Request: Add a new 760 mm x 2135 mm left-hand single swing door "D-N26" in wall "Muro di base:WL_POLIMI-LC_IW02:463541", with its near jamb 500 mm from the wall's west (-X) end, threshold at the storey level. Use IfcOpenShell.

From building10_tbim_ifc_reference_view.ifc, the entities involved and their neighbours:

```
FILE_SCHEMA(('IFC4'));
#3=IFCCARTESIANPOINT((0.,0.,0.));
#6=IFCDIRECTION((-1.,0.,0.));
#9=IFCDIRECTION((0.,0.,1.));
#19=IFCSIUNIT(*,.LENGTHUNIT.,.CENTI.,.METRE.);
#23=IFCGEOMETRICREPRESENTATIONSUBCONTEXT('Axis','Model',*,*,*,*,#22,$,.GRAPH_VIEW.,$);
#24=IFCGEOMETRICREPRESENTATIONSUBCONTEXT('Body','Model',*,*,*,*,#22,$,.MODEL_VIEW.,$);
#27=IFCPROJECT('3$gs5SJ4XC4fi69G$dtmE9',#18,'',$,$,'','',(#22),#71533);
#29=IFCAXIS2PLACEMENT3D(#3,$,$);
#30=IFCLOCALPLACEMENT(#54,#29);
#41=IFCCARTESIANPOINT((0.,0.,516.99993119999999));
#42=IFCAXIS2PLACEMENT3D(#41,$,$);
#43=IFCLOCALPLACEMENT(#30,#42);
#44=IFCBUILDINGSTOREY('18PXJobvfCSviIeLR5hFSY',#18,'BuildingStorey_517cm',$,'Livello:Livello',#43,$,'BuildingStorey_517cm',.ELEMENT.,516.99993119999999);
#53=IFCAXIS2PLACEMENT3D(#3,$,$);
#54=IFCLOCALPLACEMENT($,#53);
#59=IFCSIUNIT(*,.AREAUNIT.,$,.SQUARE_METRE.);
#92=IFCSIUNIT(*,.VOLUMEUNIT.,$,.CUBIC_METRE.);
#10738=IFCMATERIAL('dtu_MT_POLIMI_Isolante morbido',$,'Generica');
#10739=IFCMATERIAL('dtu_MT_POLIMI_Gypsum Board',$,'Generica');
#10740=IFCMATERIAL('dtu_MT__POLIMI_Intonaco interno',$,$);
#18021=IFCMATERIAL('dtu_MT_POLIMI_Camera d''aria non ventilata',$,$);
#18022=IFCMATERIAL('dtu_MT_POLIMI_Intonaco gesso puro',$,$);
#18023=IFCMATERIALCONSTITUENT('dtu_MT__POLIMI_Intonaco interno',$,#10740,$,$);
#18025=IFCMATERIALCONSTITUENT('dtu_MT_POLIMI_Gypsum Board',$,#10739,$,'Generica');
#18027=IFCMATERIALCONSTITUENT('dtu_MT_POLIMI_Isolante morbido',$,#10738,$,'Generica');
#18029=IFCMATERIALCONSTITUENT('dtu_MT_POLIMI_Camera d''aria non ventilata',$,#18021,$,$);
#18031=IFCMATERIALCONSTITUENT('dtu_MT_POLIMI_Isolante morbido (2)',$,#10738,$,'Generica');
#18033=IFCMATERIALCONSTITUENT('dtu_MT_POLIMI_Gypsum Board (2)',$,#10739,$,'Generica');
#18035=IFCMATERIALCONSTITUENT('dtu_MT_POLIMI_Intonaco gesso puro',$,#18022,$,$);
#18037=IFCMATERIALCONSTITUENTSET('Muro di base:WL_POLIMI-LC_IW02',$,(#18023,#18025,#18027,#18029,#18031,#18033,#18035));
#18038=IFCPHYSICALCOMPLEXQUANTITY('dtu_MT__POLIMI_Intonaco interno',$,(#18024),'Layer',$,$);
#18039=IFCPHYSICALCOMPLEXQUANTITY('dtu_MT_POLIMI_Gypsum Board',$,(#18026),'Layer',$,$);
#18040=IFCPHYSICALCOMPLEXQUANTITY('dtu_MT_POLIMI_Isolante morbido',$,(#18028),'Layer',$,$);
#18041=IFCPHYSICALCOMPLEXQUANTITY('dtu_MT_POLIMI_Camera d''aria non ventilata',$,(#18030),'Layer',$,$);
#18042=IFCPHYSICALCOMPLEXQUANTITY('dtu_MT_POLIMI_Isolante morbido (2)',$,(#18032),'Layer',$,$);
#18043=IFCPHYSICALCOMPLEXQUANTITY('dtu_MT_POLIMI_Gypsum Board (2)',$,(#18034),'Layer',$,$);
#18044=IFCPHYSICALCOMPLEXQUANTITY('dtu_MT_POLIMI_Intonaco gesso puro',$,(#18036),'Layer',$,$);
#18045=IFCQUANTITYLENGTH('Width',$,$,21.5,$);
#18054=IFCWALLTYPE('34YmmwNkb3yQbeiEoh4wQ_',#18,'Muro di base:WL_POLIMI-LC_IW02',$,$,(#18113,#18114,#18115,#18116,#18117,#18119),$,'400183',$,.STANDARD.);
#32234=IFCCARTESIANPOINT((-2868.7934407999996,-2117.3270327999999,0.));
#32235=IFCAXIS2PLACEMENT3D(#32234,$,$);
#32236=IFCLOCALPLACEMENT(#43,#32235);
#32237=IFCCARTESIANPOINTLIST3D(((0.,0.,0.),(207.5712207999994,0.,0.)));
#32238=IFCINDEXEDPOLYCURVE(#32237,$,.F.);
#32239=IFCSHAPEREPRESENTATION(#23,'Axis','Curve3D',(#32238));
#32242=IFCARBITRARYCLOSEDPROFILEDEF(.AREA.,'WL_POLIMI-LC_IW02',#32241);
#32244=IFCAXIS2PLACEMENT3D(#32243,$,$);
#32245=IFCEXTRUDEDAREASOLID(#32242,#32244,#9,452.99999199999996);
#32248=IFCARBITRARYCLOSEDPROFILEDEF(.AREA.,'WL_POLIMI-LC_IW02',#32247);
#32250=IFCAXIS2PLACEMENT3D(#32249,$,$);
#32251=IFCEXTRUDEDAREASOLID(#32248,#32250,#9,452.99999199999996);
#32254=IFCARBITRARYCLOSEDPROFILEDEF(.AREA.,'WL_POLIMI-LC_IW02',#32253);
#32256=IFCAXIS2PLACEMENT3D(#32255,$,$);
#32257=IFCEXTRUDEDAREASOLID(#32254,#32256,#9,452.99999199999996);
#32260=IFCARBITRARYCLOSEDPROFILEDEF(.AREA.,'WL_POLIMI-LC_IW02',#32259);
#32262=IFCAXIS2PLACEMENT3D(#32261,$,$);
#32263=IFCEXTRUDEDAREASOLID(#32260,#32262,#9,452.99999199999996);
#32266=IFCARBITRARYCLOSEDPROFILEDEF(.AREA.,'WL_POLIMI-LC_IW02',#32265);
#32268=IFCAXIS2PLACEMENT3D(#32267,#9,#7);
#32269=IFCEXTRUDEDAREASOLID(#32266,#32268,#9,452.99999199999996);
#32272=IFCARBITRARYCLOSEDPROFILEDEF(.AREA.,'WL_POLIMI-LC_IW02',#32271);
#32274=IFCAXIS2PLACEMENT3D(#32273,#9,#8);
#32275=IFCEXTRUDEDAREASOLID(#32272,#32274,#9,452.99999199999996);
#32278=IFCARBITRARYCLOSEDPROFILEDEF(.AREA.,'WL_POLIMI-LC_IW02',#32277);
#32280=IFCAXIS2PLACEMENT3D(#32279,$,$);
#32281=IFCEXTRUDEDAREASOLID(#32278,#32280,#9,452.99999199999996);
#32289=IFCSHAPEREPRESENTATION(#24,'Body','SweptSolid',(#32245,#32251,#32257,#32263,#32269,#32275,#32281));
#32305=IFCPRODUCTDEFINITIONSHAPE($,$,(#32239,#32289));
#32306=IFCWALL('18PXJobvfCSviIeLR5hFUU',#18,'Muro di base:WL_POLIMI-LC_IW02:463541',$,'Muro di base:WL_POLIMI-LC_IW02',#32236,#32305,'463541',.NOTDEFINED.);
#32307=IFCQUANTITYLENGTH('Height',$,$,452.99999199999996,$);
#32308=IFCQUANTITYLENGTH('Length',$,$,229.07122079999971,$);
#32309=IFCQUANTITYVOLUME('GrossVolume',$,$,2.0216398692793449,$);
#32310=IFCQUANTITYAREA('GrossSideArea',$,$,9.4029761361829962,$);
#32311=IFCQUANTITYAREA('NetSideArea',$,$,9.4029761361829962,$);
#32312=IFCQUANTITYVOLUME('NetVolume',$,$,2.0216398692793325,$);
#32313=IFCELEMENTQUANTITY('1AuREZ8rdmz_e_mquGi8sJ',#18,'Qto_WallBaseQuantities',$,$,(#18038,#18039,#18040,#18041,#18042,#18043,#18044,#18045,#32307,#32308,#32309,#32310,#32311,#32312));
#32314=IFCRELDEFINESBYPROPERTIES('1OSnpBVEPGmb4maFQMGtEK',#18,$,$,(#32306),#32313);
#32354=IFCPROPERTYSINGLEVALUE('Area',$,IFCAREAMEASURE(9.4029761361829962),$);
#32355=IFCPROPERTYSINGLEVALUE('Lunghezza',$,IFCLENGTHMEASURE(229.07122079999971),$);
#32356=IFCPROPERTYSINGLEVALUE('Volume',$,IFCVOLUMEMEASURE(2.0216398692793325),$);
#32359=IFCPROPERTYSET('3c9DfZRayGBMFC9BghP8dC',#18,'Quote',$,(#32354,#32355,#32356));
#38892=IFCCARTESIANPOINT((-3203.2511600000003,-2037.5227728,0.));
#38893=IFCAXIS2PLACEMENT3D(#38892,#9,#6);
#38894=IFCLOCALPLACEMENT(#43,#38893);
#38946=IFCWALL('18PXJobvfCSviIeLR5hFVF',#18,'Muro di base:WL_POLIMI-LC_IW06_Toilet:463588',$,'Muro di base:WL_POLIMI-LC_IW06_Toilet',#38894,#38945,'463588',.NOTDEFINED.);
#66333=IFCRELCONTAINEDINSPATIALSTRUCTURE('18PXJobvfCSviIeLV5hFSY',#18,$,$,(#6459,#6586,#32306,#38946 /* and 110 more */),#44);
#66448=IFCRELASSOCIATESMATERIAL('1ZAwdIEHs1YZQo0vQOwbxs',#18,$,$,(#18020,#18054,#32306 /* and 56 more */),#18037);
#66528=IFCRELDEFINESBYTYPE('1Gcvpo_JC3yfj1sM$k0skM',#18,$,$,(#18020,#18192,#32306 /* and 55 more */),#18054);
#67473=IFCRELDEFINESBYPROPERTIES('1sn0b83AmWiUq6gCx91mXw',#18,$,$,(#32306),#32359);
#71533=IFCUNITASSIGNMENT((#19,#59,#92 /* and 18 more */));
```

```python
import numpy as np
import ifcopenshell
import ifcopenshell.api.feature
import ifcopenshell.api.geometry
import ifcopenshell.api.pset
import ifcopenshell.api.root
import ifcopenshell.api.spatial
import ifcopenshell.geom
import ifcopenshell.util.element
import ifcopenshell.util.placement
import ifcopenshell.util.representation
import ifcopenshell.util.shape
import ifcopenshell.util.unit

model = ifcopenshell.open("building10_tbim_ifc_reference_view.ifc")
unit_scale = ifcopenshell.util.unit.calculate_unit_scale(model)
area_scale = ifcopenshell.util.unit.calculate_unit_scale(model, "AREAUNIT")
volume_scale = ifcopenshell.util.unit.calculate_unit_scale(model, "VOLUMEUNIT")
settings = ifcopenshell.geom.settings()


def volume(element):
    """Net volume in cubic metres, openings subtracted."""
    shape = ifcopenshell.geom.create_shape(settings, element)
    return ifcopenshell.util.shape.get_volume(shape.geometry)


wall = model.by_guid("18PXJobvfCSviIeLR5hFUU")
storey = ifcopenshell.util.element.get_container(wall, ifc_class="IfcBuildingStorey")
context = ifcopenshell.util.representation.get_context(model, "Model", "Body", "MODEL_VIEW")
before = volume(wall)

width, height, from_end, sill = 0.76, 2.135, 0.5, 0.0  # metres

# The wall runs along its own X axis, and the end named is its -X end.
wall_shape = ifcopenshell.geom.create_shape(settings, wall)
x, y, z = ifcopenshell.util.shape.get_vertices(wall_shape.geometry).T
start = x.min() + from_end
face, thickness = float(y.min()), float(y.max() - y.min())
wall_matrix = ifcopenshell.util.placement.get_local_placement(wall.ObjectPlacement)
level = ifcopenshell.util.placement.get_local_placement(storey.ObjectPlacement)[2, 3]


def in_wall(x, y):
    """Placement at x, y metres in the wall's axes, at sill height."""
    matrix = wall_matrix.copy()
    matrix[:, 3] = wall_matrix @ np.array([x / unit_scale, y / unit_scale, 0.0, 1.0])
    matrix[2, 3] = level + sill / unit_scale
    return matrix


# Opening: a box that overshoots both wall faces by 50 mm.
opening = ifcopenshell.api.root.create_entity(model, ifc_class="IfcOpeningElement", predefined_type="OPENING")
box = ifcopenshell.api.geometry.add_wall_representation(
    model, context=context, length=width, height=height, thickness=thickness + 0.1
)
ifcopenshell.api.geometry.assign_representation(model, product=opening, representation=box)
ifcopenshell.api.geometry.edit_object_placement(model, product=opening, matrix=in_wall(start, face - 0.05), is_si=False)
ifcopenshell.api.feature.add_feature(model, feature=opening, element=wall)

door = ifcopenshell.api.root.create_entity(model, ifc_class="IfcDoor", name="D-N26", predefined_type="DOOR")
door.OverallWidth, door.OverallHeight = width / unit_scale, height / unit_scale
door.OperationType = "SINGLE_SWING_LEFT"
body = ifcopenshell.api.geometry.add_door_representation(
    model,
    context=context,
    overall_width=door.OverallWidth,
    overall_height=door.OverallHeight,
    operation_type="SINGLE_SWING_LEFT",
    lining_properties={"LiningDepth": thickness / unit_scale, "ThresholdDepth": thickness / unit_scale},
)
ifcopenshell.api.geometry.assign_representation(model, product=door, representation=body)
ifcopenshell.api.spatial.assign_container(model, products=[door], relating_structure=storey)
ifcopenshell.api.feature.add_filling(model, opening=opening, element=door)

# The lining spans the wall, so the door starts at the wall face.
ifcopenshell.api.geometry.edit_object_placement(model, product=door, matrix=in_wall(start, face), is_si=False)

after = volume(wall)

# Update the wall's stored quantities.
qto = model.by_id(ifcopenshell.util.element.get_pset(wall, "Qto_WallBaseQuantities", should_inherit=False)["id"])
ifcopenshell.api.pset.edit_qto(model, qto=qto, properties={
    "NetSideArea": after / thickness / area_scale,
    "NetVolume": after / volume_scale,
})
pset = model.by_id(ifcopenshell.util.element.get_pset(wall, "Quote", should_inherit=False)["id"])
ifcopenshell.api.pset.edit_pset(model, pset=pset, properties={
    "Area": model.create_entity("IfcAreaMeasure", after / thickness / area_scale),
    "Volume": model.create_entity("IfcVolumeMeasure", after / volume_scale),
})

print(f"wall volume {before:.3f} -> {after:.3f} m3")

model.write("building10_tbim_ifc_reference_view_rev.ifc")
```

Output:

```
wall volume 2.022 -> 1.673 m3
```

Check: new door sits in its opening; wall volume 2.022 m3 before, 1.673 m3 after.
